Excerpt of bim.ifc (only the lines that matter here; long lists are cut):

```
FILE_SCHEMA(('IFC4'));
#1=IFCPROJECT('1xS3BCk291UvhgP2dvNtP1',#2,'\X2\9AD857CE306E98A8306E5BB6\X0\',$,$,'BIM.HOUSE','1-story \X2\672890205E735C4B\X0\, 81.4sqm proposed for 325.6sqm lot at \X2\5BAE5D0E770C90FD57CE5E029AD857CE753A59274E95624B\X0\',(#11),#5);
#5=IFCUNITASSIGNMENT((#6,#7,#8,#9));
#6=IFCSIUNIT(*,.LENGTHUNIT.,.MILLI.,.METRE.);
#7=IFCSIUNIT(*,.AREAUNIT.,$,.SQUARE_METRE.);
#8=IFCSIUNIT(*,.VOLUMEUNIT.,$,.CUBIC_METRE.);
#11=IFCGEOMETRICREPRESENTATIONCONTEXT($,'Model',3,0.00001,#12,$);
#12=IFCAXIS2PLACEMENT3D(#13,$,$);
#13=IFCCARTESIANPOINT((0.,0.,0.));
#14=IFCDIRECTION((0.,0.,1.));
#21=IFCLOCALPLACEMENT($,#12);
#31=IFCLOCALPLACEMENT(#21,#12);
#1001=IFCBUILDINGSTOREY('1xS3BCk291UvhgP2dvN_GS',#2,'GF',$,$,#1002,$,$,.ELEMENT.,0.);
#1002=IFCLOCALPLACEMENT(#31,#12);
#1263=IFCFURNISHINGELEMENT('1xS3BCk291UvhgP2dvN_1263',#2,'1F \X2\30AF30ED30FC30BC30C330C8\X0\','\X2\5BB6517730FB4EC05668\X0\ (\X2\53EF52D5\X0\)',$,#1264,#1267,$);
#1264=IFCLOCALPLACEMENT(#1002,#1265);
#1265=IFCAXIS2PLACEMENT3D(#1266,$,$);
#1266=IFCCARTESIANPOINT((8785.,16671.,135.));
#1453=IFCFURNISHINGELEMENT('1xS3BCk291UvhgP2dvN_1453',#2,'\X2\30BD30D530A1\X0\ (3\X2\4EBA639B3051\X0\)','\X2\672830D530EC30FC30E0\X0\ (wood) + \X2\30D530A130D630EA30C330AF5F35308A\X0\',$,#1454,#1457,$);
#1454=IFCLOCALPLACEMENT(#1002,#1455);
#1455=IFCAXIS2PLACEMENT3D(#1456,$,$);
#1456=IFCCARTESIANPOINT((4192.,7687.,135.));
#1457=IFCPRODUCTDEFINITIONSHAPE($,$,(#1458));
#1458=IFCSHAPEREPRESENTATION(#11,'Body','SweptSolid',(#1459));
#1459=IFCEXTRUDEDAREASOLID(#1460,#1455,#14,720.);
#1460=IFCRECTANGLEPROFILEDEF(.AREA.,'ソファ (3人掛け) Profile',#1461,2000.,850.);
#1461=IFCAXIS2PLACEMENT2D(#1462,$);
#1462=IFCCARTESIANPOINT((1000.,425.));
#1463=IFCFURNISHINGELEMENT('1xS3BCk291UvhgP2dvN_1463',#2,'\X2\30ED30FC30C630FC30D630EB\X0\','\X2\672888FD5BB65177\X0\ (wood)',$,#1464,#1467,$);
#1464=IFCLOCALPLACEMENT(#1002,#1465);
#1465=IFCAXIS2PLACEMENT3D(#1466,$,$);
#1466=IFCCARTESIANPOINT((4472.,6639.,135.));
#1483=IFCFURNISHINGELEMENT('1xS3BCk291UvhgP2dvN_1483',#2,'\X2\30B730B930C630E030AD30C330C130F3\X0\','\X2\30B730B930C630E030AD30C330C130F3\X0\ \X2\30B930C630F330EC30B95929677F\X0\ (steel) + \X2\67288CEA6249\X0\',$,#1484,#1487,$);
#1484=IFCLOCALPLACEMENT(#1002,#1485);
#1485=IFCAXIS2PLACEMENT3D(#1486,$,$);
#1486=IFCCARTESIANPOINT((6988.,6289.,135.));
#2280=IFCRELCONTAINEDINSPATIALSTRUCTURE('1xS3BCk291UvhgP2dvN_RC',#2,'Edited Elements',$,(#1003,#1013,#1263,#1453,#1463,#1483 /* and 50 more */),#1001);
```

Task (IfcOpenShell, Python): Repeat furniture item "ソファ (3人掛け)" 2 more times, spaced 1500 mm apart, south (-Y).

```python
import numpy as np
import ifcopenshell
import ifcopenshell.api.geometry
import ifcopenshell.api.root
import ifcopenshell.util.element
import ifcopenshell.util.placement
import ifcopenshell.util.unit

model = ifcopenshell.open("bim.ifc")
unit_scale = ifcopenshell.util.unit.calculate_unit_scale(model)


def reuse_history(source, copy):
    """copy_class also copies each property set's owner history, people and application; keep the originals."""
    for rel in copy.IsDefinedBy:
        if rel.is_a("IfcRelDefinesByProperties") and (history := rel.RelatingPropertyDefinition.OwnerHistory):
            rel.RelatingPropertyDefinition.OwnerHistory = source.OwnerHistory
            ifcopenshell.util.element.remove_deep2(model, history)


source = model.by_id(1453)
base = ifcopenshell.util.placement.get_local_placement(source.ObjectPlacement)
step = np.array([0.0, -1.0, 0.0]) * 1.5 / unit_scale

for i in range(1, 3):
    copy = ifcopenshell.api.root.copy_class(model, product=source)
    copy.Representation = ifcopenshell.util.element.copy_deep(
        model, source.Representation, exclude=["IfcGeometricRepresentationContext", "IfcRepresentationMap"]
    )
    reuse_history(source, copy)
    matrix = base.copy()
    matrix[:3, 3] += i * step
    print("added at", matrix[:3, 3].round(3) + 0.0)
    ifcopenshell.api.geometry.edit_object_placement(model, product=copy, matrix=matrix, is_si=False)

model.write("bim_v2.ifc")
```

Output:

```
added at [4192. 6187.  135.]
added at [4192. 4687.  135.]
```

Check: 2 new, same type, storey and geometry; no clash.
